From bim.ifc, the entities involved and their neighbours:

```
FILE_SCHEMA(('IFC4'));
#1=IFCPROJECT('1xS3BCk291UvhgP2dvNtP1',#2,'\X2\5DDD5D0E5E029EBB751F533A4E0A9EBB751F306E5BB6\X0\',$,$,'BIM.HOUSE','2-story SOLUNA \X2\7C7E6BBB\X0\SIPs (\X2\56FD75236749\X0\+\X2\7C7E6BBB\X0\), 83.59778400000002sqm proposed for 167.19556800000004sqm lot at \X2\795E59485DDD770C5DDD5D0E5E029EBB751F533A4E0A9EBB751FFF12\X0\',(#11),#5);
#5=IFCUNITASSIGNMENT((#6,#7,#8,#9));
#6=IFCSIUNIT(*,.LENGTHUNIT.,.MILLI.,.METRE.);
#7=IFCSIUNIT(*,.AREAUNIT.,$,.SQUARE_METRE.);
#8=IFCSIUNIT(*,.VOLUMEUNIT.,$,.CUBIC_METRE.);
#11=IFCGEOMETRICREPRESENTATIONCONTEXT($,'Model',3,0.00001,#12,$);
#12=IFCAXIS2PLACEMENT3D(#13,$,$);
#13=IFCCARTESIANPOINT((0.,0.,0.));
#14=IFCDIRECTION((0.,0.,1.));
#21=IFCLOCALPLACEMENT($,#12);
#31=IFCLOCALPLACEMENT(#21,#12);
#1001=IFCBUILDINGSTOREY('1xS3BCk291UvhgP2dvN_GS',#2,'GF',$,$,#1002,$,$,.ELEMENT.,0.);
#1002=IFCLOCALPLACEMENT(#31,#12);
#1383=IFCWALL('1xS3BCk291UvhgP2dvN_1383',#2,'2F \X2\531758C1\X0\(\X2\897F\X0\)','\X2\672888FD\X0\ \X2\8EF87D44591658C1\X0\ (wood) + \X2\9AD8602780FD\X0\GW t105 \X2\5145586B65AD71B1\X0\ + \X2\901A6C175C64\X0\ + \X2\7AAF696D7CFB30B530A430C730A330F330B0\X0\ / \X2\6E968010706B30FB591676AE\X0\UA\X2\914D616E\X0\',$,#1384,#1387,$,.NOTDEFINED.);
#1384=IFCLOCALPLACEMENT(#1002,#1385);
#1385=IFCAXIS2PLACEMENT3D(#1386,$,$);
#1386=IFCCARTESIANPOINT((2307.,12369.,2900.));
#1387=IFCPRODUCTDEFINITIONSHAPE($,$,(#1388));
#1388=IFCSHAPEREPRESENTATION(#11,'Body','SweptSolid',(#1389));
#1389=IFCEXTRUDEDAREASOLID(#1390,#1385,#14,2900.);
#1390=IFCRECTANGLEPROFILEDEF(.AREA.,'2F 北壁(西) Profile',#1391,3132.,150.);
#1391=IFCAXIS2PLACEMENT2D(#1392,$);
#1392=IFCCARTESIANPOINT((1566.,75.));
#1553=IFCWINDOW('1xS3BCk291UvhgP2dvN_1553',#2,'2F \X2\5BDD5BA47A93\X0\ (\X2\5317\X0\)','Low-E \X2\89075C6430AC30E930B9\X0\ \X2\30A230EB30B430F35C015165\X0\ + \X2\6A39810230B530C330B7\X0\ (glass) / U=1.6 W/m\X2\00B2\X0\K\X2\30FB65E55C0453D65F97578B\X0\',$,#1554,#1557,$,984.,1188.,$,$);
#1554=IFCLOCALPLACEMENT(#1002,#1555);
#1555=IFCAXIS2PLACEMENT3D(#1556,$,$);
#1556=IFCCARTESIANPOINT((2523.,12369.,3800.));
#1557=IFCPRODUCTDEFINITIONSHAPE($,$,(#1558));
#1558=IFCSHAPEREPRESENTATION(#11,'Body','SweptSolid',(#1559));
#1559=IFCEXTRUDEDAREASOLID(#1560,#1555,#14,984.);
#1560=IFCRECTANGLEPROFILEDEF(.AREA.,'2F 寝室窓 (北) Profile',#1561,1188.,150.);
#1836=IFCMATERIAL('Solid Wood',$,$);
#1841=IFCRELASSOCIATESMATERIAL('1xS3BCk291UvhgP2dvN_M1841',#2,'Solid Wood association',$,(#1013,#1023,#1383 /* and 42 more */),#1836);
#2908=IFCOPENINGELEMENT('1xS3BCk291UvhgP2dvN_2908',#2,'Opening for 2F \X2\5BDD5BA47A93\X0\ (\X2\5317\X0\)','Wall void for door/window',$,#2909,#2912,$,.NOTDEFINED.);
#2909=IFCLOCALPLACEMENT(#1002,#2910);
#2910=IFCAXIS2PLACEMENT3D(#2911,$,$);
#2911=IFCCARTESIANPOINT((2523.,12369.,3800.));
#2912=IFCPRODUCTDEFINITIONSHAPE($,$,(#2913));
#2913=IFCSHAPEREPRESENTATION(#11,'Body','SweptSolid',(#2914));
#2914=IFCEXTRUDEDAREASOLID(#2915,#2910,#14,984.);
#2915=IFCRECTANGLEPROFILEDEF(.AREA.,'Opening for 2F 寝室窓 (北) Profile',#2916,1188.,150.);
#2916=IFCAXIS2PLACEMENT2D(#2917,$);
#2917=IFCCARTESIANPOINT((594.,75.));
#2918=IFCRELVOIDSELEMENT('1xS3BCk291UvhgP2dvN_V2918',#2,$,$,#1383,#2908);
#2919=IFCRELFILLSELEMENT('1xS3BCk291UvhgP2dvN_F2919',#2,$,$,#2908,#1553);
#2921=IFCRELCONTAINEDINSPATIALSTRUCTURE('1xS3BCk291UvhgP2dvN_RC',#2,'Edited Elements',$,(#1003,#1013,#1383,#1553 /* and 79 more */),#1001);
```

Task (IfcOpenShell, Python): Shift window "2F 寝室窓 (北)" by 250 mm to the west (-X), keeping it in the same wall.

```python
import ifcopenshell
import ifcopenshell.api.geometry
import ifcopenshell.util.placement

model = ifcopenshell.open("bim.ifc")

window = model.by_id(1553)
opening = window.FillsVoids[0].RelatingOpeningElement
wall = opening.VoidsElements[0].RelatingBuildingElement

wall_matrix = ifcopenshell.util.placement.get_local_placement(wall.ObjectPlacement)
shift = wall_matrix[:3, 0] * -250.0
before = ifcopenshell.util.placement.get_local_placement(window.ObjectPlacement)[:3, 3].copy()

# The window is not placed relative to its opening, so move both.
for product in (opening, window):
    matrix = ifcopenshell.util.placement.get_local_placement(product.ObjectPlacement)
    matrix[:3, 3] += shift
    ifcopenshell.api.geometry.edit_object_placement(model, product=product, matrix=matrix, is_si=False)

after = ifcopenshell.util.placement.get_local_placement(window.ObjectPlacement)[:3, 3]
print("window moved by", (after - before).round(3) + 0.0)

model.write("bim-out.ifc")
```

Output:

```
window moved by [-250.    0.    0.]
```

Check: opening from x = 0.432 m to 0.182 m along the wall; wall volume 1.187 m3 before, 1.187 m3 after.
